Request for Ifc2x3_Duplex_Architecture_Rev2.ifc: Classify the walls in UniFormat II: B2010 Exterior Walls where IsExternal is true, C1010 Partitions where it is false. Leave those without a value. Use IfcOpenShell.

First a look at what the model holds.

```python
import ifcopenshell
import ifcopenshell.util.element

model = ifcopenshell.open("Ifc2x3_Duplex_Architecture_Rev2.ifc")
print(model.schema)
print("classifications:", [c.Name for c in model.by_type("IfcClassification")])
values = [ifcopenshell.util.element.get_pset(e, "Pset_WallCommon", "IsExternal") for e in model.by_type("IfcWall")]
for value in (True, False, None):
    print("IsExternal", value, values.count(value))
```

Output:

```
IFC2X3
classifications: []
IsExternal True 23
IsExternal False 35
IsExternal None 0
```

```python
import ifcopenshell
import ifcopenshell.api.classification
import ifcopenshell.util.element

model = ifcopenshell.open("Ifc2x3_Duplex_Architecture_Rev2.ifc")

# IFC2X3 requires Source and Edition and has no link from the project to the system.
system = model.create_entity("IfcClassification", Source="ASTM", Edition="E1557", Name="UniFormat II")

walls = model.by_type("IfcWall")
external = {e: ifcopenshell.util.element.get_pset(e, "Pset_WallCommon", "IsExternal") for e in walls}
for flag, code, name in ((True, "B2010", "Exterior Walls"), (False, "C1010", "Partitions")):
    products = [e for e in walls if external[e] is flag]
    ifcopenshell.api.classification.add_reference(
        model, products=products, classification=system, identification=code, name=name
    )
    print(code, len(products))

model.write("Ifc2x3_Duplex_Architecture_Rev2_updated.ifc")
```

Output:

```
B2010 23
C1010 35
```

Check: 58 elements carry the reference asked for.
